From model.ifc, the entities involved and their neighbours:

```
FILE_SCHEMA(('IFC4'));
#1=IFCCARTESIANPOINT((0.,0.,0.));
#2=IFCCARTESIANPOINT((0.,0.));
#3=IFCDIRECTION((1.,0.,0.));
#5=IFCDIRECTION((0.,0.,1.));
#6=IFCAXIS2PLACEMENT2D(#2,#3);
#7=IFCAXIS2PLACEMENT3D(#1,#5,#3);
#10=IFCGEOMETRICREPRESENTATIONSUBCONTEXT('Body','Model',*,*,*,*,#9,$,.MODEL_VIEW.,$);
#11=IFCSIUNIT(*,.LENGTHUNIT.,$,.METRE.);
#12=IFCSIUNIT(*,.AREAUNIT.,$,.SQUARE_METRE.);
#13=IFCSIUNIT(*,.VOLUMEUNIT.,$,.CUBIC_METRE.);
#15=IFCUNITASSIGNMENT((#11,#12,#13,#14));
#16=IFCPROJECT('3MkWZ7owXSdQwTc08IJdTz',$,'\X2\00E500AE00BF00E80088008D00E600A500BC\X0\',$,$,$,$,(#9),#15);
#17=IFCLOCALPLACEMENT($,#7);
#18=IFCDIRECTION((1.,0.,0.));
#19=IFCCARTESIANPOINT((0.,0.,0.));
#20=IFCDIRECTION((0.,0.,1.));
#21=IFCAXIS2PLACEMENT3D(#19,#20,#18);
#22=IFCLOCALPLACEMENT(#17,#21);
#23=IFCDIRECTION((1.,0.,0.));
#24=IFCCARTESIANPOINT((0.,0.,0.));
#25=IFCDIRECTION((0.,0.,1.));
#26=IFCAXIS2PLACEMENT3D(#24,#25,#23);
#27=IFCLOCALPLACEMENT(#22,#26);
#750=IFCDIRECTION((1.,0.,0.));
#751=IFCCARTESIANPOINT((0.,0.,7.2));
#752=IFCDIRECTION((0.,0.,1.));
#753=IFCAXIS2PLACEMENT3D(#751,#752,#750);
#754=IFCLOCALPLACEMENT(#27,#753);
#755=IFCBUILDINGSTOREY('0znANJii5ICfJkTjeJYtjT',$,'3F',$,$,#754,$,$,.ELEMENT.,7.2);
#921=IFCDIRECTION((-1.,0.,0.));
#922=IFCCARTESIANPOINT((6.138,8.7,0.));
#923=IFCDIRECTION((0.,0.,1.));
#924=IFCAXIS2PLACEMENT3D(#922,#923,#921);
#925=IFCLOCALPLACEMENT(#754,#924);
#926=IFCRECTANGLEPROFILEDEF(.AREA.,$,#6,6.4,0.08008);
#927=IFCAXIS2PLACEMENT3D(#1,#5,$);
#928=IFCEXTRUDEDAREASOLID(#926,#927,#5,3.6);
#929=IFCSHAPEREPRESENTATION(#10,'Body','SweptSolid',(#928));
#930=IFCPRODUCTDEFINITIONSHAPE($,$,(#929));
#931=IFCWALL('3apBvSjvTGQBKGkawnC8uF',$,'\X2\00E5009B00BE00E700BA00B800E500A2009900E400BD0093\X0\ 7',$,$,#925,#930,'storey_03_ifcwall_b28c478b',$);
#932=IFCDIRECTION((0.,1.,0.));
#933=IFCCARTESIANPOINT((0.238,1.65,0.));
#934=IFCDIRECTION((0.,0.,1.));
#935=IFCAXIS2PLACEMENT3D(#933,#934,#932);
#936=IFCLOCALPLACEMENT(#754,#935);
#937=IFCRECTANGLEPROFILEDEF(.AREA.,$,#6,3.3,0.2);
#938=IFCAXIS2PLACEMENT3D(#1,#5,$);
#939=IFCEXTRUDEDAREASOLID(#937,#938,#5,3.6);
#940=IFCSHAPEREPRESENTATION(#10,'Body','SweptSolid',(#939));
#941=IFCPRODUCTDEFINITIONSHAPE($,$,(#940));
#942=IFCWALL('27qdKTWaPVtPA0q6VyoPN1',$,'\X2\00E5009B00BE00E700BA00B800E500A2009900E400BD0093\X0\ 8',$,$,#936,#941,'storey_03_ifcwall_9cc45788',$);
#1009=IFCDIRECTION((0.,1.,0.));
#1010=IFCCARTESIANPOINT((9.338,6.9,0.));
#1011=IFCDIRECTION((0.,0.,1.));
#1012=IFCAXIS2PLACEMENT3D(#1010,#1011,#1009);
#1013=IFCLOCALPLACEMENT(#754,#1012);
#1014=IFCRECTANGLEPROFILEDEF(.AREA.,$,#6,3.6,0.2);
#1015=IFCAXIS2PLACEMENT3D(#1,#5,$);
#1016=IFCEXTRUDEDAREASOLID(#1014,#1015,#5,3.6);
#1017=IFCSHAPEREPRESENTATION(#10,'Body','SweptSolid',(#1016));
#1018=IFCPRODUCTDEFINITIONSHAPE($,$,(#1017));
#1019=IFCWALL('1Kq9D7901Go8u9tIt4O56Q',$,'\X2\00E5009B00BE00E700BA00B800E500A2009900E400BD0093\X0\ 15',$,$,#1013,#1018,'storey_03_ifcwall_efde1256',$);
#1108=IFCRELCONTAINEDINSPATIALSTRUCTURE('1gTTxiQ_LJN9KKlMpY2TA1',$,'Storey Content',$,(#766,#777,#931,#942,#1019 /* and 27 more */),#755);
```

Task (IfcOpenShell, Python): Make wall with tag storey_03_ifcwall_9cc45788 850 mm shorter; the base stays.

```python
import ifcopenshell
import ifcopenshell.geom
import ifcopenshell.util.representation
import ifcopenshell.util.shape
import ifcopenshell.util.unit

model = ifcopenshell.open("model.ifc")
unit_scale = ifcopenshell.util.unit.calculate_unit_scale(model)
settings = ifcopenshell.geom.settings()


def volume(element):
    """Net volume in cubic metres, openings subtracted."""
    shape = ifcopenshell.geom.create_shape(settings, element)
    return ifcopenshell.util.shape.get_volume(shape.geometry)


wall = model.by_guid("27qdKTWaPVtPA0q6VyoPN1")
before = volume(wall)

body = ifcopenshell.util.representation.get_representation(wall, "Model", "Body")
solid = body.Items[0]
old_height = solid.Depth
solid.Depth -= 0.85 / unit_scale
after = volume(wall)

print(f"height {old_height:g} -> {solid.Depth:g}, volume {before:.3f} -> {after:.3f} m3")

model.write("model_updated.ifc")
```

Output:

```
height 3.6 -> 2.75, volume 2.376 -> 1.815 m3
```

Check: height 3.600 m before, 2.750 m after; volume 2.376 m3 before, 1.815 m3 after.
